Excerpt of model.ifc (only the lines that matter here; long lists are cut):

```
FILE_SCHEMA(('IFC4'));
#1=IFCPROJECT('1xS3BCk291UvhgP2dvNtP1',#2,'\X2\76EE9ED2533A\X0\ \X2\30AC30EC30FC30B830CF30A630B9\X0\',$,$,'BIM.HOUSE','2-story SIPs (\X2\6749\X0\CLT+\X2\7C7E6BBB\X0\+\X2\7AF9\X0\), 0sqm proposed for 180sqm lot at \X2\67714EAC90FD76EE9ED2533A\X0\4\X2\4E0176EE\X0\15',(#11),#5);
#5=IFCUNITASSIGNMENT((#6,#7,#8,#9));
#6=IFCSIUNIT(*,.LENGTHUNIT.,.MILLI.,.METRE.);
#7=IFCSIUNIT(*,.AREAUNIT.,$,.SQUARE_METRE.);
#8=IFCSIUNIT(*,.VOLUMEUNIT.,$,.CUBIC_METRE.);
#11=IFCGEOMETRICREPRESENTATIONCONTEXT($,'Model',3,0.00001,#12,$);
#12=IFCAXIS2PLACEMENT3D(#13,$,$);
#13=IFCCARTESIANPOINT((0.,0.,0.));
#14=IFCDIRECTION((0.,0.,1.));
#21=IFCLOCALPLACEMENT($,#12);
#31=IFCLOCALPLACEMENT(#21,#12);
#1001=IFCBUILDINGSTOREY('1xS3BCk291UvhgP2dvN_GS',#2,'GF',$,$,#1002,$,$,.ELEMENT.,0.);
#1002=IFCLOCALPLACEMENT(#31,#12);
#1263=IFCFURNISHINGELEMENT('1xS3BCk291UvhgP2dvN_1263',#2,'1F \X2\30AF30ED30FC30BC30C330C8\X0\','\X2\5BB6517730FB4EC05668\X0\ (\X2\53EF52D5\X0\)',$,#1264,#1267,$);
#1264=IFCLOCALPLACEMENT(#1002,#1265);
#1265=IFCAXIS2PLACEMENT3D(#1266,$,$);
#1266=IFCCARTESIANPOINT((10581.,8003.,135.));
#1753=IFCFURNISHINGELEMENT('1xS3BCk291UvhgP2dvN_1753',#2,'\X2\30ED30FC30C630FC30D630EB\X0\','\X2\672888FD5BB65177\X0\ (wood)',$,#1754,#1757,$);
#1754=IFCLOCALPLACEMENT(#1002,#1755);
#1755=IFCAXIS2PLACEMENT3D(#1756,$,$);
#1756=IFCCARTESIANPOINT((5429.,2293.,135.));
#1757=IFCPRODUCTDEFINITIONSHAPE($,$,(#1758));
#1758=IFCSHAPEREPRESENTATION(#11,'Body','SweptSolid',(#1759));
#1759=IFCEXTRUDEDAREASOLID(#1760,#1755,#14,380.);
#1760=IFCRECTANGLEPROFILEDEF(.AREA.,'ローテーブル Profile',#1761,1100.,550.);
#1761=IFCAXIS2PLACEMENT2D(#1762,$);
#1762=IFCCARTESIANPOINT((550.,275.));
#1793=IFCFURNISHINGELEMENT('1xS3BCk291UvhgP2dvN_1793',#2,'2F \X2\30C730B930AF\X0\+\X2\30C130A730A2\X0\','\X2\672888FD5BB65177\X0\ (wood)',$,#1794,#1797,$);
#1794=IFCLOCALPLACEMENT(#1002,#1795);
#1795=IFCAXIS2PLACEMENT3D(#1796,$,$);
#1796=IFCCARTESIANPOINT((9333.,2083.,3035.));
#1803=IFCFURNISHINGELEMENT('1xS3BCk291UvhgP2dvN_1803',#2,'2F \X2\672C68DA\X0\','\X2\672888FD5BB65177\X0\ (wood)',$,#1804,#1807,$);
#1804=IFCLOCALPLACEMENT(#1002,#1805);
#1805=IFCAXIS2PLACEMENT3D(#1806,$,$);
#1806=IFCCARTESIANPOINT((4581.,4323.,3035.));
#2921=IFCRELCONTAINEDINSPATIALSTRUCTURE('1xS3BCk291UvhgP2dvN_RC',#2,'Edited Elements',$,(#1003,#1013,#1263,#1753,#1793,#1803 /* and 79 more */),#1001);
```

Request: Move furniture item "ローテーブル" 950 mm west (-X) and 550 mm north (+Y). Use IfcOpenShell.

```python
import ifcopenshell
import ifcopenshell.api.geometry
import ifcopenshell.util.placement

model = ifcopenshell.open("model.ifc")

item = model.by_guid("1xS3BCk291UvhgP2dvN_1753")
matrix = ifcopenshell.util.placement.get_local_placement(item.ObjectPlacement)
matrix[0, 3] -= 950.0
matrix[1, 3] += 550.0
ifcopenshell.api.geometry.edit_object_placement(model, product=item, matrix=matrix, is_si=False)

print(ifcopenshell.util.placement.get_local_placement(item.ObjectPlacement).round(3) + 0.0)

model.write("model_v2.ifc")
```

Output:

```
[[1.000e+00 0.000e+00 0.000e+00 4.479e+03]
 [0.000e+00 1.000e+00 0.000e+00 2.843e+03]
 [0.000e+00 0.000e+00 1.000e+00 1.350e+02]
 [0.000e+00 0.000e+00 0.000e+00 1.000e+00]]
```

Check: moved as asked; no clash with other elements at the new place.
